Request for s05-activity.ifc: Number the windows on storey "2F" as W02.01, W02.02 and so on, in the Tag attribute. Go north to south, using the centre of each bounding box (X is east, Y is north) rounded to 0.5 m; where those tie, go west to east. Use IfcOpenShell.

First a look at what the model holds.

```python
import ifcopenshell
import ifcopenshell.util.element
import ifcopenshell.util.placement

model = ifcopenshell.open("s05-activity.ifc")
print(model.schema)
storey = next(s for s in model.by_type("IfcBuildingStorey") if s.Name == "2F")
windows = [e for e in ifcopenshell.util.element.get_decomposition(storey) if e.is_a("IfcWindow")]
for e in sorted(windows, key=lambda e: e.id()):
    origin = ifcopenshell.util.placement.get_local_placement(e.ObjectPlacement)[:3, 3]
    print(e.id(), e.Tag, e.Name, origin.round(2) + 0.0, sep=" | ")
```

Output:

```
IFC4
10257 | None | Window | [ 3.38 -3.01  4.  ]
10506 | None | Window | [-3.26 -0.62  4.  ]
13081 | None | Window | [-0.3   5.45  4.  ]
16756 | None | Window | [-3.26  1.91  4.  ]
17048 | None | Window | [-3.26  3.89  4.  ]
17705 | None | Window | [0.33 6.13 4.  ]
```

```python
import ifcopenshell
import ifcopenshell.geom
import ifcopenshell.util.element
import ifcopenshell.util.shape

model = ifcopenshell.open("s05-activity.ifc")
settings = ifcopenshell.geom.settings()
settings.set("use-world-coords", True)


def centre(element):
    shape = ifcopenshell.geom.create_shape(settings, element)
    return ifcopenshell.util.shape.get_bbox_centroid(shape.geometry)


storey = next(s for s in model.by_type("IfcBuildingStorey") if s.Name == "2F")
windows = [e for e in ifcopenshell.util.element.get_decomposition(storey) if e.is_a("IfcWindow")]

# Insertion points can sit at a corner or the storey origin, so sort by the geometry (in metres).
centres = {e: centre(e) for e in windows}
windows.sort(key=lambda e: (-round(centres[e][1] / 0.5), centres[e][0]))

for i, e in enumerate(windows, start=1):
    number = f"W02.{i:02d}"
    e.Tag = number
    print(e.id(), number)

model.write("s05-activity_rev.ifc")
```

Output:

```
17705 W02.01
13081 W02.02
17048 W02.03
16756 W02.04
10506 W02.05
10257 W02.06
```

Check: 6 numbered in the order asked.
